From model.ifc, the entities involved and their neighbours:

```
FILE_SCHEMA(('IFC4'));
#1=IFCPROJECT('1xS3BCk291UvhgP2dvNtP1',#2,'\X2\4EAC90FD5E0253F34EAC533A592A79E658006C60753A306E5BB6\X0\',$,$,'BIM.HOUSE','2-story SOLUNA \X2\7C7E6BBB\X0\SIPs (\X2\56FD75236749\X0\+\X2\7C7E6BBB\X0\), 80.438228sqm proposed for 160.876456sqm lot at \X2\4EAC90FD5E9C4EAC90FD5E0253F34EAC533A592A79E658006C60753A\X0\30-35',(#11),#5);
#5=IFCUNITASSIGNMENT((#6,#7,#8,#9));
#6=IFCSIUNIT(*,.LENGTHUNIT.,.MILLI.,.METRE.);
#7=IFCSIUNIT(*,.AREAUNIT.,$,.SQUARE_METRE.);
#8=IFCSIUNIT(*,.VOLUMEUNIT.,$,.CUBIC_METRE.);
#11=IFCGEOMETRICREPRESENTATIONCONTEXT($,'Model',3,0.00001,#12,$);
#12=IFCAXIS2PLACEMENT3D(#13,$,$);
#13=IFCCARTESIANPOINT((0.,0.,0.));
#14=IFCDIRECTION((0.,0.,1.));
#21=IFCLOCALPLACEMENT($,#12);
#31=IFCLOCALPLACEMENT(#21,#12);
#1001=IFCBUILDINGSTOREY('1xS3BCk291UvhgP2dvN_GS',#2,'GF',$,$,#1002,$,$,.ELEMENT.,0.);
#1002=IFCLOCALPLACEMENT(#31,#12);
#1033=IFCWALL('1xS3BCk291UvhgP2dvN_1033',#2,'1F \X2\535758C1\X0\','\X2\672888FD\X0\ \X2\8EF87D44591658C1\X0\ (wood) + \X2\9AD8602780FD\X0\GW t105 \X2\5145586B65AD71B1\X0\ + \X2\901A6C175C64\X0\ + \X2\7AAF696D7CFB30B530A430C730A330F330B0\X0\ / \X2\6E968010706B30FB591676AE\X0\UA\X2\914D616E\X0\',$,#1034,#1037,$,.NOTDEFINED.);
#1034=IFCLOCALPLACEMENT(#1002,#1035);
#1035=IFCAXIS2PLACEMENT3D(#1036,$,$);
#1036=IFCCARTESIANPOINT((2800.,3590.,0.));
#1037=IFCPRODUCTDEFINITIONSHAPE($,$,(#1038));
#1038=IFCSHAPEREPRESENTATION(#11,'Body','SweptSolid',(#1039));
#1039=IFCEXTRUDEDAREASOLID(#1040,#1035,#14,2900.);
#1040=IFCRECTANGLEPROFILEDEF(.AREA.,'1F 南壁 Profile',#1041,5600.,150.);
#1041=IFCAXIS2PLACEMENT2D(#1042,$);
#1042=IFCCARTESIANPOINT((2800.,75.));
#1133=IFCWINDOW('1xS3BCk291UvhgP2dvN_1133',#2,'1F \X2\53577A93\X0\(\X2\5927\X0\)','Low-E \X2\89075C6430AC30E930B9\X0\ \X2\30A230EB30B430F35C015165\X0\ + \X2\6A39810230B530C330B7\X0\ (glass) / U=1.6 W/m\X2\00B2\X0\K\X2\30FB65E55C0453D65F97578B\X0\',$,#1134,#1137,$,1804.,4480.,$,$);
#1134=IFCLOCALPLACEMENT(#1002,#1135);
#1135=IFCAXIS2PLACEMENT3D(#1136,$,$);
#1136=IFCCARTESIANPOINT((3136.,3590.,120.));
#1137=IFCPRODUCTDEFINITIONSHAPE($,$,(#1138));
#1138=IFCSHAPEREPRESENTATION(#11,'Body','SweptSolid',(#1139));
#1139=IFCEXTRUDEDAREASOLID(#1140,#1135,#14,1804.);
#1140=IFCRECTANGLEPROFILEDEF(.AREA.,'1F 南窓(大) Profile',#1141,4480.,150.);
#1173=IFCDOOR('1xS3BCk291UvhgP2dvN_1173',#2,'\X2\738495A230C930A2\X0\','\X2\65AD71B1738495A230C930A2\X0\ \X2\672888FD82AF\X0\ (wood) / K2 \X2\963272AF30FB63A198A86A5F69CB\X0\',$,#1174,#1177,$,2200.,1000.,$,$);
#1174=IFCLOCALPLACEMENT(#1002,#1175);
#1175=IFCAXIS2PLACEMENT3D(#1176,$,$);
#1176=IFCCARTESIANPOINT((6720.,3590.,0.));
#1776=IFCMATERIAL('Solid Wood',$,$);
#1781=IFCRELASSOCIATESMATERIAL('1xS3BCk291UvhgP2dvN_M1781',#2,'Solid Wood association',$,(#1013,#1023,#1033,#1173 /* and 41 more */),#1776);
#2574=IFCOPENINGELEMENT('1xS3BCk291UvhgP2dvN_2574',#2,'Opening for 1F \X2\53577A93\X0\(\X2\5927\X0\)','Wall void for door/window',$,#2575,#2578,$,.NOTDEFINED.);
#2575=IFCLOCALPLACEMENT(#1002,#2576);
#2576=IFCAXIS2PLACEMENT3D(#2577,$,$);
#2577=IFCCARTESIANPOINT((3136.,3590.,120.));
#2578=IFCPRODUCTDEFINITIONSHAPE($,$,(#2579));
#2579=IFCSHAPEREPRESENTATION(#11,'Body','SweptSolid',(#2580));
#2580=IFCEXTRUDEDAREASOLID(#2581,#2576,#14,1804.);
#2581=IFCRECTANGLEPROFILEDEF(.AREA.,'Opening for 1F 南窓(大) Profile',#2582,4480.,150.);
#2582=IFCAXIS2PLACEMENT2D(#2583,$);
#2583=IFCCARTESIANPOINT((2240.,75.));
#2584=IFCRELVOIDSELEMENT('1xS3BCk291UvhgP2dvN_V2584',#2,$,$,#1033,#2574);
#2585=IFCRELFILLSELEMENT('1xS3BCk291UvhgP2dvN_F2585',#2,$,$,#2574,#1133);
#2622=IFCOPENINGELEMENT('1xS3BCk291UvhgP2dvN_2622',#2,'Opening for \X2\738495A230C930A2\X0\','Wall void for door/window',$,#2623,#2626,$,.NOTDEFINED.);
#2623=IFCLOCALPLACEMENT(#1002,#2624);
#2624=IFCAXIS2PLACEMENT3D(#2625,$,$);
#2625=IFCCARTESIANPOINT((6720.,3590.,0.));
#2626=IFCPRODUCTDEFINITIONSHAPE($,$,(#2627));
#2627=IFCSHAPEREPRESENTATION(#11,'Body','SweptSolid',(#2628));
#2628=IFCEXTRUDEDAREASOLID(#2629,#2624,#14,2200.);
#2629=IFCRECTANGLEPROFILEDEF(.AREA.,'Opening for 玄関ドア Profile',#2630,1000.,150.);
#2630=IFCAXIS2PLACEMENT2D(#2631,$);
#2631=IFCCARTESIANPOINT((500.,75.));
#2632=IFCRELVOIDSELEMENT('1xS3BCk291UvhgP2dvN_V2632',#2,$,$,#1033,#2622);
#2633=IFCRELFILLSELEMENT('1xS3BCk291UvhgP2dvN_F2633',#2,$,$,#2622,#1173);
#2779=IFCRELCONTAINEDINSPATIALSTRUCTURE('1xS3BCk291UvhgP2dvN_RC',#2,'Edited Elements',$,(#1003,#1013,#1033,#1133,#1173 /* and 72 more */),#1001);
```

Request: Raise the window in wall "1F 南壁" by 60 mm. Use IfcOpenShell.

```python
import numpy as np
import ifcopenshell
import ifcopenshell.api.geometry
import ifcopenshell.util.placement
import ifcopenshell.util.unit

model = ifcopenshell.open("model.ifc")
unit_scale = ifcopenshell.util.unit.calculate_unit_scale(model)

window = model.by_guid("1xS3BCk291UvhgP2dvN_1133")
opening = window.FillsVoids[0].RelatingOpeningElement
dz = 0.06 / unit_scale

shift = np.array([0.0, 0.0, dz])
# The window is not placed relative to its opening, so move both.
for product in (opening, window):
    matrix = ifcopenshell.util.placement.get_local_placement(product.ObjectPlacement)
    matrix[:3, 3] += shift
    ifcopenshell.api.geometry.edit_object_placement(model, product=product, matrix=matrix, is_si=False)

print(f"moved by {dz * unit_scale:+.3f} m")

model.write("model_edited.ifc")
```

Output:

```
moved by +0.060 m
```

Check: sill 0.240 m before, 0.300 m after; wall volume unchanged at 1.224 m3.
